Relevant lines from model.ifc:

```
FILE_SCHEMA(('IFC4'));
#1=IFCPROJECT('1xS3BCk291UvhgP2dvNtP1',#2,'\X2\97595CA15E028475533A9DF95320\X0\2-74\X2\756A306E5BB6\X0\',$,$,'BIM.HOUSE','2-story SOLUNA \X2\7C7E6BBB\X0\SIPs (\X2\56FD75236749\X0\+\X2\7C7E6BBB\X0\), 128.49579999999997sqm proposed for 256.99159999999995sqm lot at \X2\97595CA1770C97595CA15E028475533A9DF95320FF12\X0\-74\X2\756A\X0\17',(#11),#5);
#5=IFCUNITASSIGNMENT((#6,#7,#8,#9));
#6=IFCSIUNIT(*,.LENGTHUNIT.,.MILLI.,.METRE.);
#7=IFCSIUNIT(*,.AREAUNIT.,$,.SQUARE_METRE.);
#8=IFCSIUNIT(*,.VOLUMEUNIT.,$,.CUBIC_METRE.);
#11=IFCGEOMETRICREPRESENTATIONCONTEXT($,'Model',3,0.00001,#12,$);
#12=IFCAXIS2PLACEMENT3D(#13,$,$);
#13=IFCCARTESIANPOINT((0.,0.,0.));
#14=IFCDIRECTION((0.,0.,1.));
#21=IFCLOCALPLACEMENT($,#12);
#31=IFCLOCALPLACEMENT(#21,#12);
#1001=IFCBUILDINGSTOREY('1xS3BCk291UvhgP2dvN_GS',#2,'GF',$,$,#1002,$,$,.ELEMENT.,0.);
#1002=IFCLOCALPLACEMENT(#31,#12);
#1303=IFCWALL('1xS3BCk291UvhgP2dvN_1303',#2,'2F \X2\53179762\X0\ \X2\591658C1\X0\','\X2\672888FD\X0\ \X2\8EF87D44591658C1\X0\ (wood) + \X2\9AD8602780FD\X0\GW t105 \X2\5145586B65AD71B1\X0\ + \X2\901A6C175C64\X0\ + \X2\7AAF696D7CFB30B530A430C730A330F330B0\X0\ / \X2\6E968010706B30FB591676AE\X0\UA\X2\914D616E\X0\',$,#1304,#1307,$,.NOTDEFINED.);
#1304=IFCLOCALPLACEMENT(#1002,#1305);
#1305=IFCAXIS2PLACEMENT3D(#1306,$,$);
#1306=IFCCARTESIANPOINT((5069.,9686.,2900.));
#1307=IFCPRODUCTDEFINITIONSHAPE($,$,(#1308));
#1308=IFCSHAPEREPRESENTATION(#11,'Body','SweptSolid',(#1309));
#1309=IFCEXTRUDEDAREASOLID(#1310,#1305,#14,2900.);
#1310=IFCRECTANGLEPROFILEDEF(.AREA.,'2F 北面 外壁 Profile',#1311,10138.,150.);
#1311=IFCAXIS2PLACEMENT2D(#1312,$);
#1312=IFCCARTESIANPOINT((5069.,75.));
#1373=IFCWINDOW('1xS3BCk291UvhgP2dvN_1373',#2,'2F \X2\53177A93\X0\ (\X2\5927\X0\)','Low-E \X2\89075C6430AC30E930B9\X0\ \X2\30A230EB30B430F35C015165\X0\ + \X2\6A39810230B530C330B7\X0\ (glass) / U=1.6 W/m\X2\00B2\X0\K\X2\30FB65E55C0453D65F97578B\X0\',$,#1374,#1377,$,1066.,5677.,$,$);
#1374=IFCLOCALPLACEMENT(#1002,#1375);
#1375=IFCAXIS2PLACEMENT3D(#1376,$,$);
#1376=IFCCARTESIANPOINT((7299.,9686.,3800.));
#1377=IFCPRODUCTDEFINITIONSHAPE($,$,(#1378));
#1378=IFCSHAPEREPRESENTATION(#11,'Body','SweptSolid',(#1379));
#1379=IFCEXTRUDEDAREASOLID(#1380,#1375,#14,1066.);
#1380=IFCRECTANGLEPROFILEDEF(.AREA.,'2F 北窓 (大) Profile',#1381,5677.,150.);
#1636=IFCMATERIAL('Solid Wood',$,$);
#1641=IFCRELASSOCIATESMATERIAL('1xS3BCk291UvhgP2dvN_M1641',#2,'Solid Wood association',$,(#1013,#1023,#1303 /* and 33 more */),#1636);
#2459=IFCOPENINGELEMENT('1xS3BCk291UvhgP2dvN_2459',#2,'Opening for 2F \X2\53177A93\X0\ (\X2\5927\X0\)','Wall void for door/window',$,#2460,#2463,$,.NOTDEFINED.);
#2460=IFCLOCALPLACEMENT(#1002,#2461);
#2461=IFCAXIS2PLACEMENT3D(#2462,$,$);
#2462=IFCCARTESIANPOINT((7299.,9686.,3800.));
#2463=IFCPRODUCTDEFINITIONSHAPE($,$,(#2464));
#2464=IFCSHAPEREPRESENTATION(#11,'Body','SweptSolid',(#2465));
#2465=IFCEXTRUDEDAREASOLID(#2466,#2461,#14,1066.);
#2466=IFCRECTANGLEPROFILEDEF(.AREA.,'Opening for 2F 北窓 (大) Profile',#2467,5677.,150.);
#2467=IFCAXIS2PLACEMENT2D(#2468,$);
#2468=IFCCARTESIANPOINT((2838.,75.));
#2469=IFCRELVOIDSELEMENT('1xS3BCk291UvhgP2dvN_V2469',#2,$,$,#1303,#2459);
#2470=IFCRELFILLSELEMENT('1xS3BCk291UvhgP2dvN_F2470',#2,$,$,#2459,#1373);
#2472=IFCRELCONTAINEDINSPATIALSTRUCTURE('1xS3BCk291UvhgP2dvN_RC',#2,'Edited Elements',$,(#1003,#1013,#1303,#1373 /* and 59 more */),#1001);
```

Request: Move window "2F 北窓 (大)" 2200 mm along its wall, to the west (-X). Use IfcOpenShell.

```python
import ifcopenshell
import ifcopenshell.api.geometry
import ifcopenshell.util.placement
import ifcopenshell.util.unit

model = ifcopenshell.open("model.ifc")
unit_scale = ifcopenshell.util.unit.calculate_unit_scale(model)

window = model.by_guid("1xS3BCk291UvhgP2dvN_1373")
opening = window.FillsVoids[0].RelatingOpeningElement
wall = opening.VoidsElements[0].RelatingBuildingElement

wall_matrix = ifcopenshell.util.placement.get_local_placement(wall.ObjectPlacement)
shift = wall_matrix[:3, 0] * -2.2 / unit_scale
before = ifcopenshell.util.placement.get_local_placement(window.ObjectPlacement)[:3, 3].copy()

# The window is not placed relative to its opening, so move both.
for product in (opening, window):
    matrix = ifcopenshell.util.placement.get_local_placement(product.ObjectPlacement)
    matrix[:3, 3] += shift
    ifcopenshell.api.geometry.edit_object_placement(model, product=product, matrix=matrix, is_si=False)

after = ifcopenshell.util.placement.get_local_placement(window.ObjectPlacement)[:3, 3]
print("window moved by", (after - before).round(3) + 0.0)

model.write("model_v2.ifc")
```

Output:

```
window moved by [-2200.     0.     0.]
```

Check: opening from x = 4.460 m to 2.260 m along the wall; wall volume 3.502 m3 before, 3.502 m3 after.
